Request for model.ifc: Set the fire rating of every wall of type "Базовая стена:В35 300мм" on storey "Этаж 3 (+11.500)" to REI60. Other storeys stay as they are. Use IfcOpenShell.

First a look at what the model holds.

```python
import ifcopenshell
import ifcopenshell.util.element

model = ifcopenshell.open("model.ifc")
print(model.schema)
storey = next(s for s in model.by_type("IfcBuildingStorey") if s.Name == "Этаж 3 (+11.500)")
walls = [e for e in ifcopenshell.util.element.get_decomposition(storey) if e.is_a("IfcWall")]
seen = {}
for e in walls:
    element_type = ifcopenshell.util.element.get_type(e)
    key = (element_type.Name if element_type != e and element_type else None, ifcopenshell.util.element.get_pset(e, "Pset_WallCommon", "FireRating"))
    seen[key] = seen.get(key, 0) + 1
for (name, value), count in sorted(seen.items(), key=str):
    print(count, "x", name, "|", value)
```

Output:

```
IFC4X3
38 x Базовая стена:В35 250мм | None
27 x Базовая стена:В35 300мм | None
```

```python
import ifcopenshell
import ifcopenshell.api.pset
import ifcopenshell.util.element

model = ifcopenshell.open("model.ifc")

storey = next(s for s in model.by_type("IfcBuildingStorey") if s.Name == "Этаж 3 (+11.500)")
walls = [e for e in ifcopenshell.util.element.get_decomposition(storey) if e.is_a("IfcWall")]

count = 0
for e in walls:
    element_type = ifcopenshell.util.element.get_type(e)
    if element_type in (None, e) or element_type.Name != "Базовая стена:В35 300мм":
        continue
    # add_pset returns the element's existing set when there is one.
    pset = ifcopenshell.api.pset.add_pset(model, product=e, name="Pset_WallCommon")
    ifcopenshell.api.pset.edit_pset(model, pset=pset, properties={"FireRating": "REI60"})
    count += 1

print(count, "walls updated")

model.write("model_rev.ifc")
```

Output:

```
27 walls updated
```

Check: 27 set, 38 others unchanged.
